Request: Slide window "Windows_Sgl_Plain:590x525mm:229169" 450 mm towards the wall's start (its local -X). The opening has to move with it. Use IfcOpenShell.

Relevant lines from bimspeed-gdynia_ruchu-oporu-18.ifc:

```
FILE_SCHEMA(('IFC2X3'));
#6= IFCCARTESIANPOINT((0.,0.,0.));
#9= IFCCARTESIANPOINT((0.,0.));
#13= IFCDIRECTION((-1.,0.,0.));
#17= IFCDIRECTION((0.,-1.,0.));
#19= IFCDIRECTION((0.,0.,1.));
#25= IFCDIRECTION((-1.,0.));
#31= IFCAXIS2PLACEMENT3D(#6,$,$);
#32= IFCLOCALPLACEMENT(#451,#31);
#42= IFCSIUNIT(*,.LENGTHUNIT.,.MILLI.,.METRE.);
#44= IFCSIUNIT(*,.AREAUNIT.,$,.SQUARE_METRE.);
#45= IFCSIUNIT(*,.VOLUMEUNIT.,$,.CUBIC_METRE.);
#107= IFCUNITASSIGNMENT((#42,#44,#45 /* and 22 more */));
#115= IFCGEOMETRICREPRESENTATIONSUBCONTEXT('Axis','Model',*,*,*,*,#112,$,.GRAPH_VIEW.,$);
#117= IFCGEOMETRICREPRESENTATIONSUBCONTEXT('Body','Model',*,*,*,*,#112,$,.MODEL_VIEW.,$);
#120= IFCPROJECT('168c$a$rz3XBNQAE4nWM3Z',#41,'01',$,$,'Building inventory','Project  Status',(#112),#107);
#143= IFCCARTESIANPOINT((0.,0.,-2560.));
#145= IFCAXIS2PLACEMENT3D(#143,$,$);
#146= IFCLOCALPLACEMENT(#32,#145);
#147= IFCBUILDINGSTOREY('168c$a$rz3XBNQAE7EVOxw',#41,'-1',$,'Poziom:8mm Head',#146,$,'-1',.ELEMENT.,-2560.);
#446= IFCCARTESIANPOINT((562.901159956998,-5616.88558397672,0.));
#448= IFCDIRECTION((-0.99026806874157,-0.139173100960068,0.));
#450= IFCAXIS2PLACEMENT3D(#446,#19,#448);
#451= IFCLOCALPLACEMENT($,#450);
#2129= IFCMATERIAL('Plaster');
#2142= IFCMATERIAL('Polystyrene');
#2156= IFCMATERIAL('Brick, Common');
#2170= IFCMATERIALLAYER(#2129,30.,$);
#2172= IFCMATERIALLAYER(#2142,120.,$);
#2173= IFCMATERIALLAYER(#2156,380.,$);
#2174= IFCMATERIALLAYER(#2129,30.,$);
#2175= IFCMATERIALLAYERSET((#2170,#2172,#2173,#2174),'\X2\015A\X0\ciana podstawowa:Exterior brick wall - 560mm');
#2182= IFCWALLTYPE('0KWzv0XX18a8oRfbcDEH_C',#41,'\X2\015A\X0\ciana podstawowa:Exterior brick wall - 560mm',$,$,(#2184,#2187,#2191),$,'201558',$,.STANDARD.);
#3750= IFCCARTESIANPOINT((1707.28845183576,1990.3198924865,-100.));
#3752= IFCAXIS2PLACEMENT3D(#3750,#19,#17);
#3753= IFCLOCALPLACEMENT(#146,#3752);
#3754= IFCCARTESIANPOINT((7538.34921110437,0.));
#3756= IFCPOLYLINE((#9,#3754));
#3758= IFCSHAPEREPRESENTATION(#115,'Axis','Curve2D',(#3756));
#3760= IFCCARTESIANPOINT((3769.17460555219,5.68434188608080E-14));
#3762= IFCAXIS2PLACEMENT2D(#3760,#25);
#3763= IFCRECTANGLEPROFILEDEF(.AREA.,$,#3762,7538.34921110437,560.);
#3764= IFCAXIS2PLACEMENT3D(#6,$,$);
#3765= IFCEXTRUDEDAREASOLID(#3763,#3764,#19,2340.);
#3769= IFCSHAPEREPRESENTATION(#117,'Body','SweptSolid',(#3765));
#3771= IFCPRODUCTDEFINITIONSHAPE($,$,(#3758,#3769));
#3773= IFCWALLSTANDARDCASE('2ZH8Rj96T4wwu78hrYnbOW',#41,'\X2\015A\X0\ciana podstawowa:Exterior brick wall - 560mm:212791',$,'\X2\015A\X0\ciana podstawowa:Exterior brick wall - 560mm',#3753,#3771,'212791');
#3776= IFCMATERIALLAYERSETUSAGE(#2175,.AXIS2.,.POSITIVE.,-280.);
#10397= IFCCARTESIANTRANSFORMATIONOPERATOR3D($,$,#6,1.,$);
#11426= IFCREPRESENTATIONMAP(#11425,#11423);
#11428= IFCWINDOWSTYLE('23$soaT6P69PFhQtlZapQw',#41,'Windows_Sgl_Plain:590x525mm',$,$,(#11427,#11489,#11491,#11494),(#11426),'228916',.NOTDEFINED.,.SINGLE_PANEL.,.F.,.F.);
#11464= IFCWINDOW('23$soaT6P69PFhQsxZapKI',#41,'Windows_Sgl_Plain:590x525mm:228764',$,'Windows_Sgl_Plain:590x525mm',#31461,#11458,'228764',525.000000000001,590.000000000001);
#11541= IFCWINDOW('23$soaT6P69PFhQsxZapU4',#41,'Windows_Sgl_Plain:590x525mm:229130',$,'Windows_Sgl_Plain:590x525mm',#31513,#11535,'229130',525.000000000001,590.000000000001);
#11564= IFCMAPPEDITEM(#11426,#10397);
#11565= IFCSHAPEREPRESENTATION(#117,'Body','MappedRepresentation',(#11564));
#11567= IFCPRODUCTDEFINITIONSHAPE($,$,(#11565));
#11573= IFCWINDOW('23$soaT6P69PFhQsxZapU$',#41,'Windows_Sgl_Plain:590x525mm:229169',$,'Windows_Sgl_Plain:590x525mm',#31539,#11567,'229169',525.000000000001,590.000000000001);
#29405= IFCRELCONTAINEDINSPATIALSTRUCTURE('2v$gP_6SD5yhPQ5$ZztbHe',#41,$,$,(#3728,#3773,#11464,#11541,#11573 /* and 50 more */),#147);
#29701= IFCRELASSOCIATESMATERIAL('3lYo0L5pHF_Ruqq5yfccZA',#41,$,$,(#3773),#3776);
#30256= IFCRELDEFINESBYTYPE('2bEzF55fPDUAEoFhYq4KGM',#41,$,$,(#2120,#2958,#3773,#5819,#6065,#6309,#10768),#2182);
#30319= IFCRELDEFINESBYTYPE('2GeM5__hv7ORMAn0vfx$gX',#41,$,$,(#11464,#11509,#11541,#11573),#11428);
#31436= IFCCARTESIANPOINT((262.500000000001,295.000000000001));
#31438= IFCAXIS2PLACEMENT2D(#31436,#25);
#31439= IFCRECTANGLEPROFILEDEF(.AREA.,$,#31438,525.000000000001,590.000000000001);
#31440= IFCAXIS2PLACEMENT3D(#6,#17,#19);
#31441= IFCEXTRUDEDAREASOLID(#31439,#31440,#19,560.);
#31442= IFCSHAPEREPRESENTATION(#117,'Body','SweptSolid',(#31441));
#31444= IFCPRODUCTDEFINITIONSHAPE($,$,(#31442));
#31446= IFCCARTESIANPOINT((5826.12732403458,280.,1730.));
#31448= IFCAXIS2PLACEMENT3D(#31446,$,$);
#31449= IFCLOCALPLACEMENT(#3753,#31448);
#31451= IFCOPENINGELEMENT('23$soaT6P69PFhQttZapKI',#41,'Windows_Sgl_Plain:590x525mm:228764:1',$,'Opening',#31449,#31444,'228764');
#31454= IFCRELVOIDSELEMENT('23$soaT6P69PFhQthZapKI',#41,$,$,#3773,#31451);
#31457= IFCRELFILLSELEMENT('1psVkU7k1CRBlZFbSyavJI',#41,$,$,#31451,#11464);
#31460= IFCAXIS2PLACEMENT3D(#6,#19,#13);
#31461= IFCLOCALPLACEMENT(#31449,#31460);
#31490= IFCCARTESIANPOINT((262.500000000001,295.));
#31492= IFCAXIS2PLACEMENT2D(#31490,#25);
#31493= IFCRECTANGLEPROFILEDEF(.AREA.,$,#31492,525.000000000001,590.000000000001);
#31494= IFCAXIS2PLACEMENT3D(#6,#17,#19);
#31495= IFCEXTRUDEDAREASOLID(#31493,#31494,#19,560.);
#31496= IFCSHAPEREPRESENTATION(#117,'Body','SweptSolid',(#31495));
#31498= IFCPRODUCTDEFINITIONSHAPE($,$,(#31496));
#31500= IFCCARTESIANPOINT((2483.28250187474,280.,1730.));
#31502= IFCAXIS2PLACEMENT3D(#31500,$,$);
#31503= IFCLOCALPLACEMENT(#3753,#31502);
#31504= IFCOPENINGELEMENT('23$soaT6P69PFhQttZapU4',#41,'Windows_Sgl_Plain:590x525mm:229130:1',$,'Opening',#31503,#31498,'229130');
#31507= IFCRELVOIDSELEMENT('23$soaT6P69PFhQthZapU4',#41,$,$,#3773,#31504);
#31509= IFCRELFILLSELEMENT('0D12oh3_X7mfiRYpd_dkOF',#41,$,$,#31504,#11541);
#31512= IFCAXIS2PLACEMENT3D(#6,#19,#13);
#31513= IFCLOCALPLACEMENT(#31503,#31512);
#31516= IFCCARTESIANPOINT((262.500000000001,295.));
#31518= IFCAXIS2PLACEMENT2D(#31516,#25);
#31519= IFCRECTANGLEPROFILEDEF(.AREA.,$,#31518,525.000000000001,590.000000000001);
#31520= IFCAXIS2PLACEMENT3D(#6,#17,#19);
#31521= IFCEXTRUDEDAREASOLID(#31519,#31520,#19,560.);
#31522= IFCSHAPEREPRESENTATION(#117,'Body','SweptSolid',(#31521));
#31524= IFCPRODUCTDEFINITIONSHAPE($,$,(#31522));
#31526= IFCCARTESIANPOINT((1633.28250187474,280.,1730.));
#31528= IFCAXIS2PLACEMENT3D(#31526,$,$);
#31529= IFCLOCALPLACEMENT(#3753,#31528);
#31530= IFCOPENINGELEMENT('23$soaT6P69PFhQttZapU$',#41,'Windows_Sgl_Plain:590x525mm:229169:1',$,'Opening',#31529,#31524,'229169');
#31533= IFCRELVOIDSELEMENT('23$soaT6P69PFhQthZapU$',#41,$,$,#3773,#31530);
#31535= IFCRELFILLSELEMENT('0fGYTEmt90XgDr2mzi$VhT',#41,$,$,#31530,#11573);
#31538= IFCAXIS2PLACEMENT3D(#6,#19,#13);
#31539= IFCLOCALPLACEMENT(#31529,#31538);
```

```python
import ifcopenshell
import ifcopenshell.api.geometry
import ifcopenshell.util.placement

model = ifcopenshell.open("bimspeed-gdynia_ruchu-oporu-18.ifc")

window = model.by_id(11573)
opening = window.FillsVoids[0].RelatingOpeningElement
wall = opening.VoidsElements[0].RelatingBuildingElement

wall_matrix = ifcopenshell.util.placement.get_local_placement(wall.ObjectPlacement)
shift = wall_matrix[:3, 0] * -450.0
before = ifcopenshell.util.placement.get_local_placement(window.ObjectPlacement)[:3, 3].copy()

# The window is placed relative to its opening, so it follows when the opening moves.
matrix = ifcopenshell.util.placement.get_local_placement(opening.ObjectPlacement)
matrix[:3, 3] += shift
ifcopenshell.api.geometry.edit_object_placement(
    model, product=opening, matrix=matrix, is_si=False, should_transform_children=True
)

after = ifcopenshell.util.placement.get_local_placement(window.ObjectPlacement)[:3, 3]
print("window moved by", (after - before).round(3) + 0.0)

model.write("bimspeed-gdynia_ruchu-oporu-18_rev.ifc")
```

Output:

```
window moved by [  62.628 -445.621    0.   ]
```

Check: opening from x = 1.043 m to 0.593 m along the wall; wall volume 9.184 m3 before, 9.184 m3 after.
